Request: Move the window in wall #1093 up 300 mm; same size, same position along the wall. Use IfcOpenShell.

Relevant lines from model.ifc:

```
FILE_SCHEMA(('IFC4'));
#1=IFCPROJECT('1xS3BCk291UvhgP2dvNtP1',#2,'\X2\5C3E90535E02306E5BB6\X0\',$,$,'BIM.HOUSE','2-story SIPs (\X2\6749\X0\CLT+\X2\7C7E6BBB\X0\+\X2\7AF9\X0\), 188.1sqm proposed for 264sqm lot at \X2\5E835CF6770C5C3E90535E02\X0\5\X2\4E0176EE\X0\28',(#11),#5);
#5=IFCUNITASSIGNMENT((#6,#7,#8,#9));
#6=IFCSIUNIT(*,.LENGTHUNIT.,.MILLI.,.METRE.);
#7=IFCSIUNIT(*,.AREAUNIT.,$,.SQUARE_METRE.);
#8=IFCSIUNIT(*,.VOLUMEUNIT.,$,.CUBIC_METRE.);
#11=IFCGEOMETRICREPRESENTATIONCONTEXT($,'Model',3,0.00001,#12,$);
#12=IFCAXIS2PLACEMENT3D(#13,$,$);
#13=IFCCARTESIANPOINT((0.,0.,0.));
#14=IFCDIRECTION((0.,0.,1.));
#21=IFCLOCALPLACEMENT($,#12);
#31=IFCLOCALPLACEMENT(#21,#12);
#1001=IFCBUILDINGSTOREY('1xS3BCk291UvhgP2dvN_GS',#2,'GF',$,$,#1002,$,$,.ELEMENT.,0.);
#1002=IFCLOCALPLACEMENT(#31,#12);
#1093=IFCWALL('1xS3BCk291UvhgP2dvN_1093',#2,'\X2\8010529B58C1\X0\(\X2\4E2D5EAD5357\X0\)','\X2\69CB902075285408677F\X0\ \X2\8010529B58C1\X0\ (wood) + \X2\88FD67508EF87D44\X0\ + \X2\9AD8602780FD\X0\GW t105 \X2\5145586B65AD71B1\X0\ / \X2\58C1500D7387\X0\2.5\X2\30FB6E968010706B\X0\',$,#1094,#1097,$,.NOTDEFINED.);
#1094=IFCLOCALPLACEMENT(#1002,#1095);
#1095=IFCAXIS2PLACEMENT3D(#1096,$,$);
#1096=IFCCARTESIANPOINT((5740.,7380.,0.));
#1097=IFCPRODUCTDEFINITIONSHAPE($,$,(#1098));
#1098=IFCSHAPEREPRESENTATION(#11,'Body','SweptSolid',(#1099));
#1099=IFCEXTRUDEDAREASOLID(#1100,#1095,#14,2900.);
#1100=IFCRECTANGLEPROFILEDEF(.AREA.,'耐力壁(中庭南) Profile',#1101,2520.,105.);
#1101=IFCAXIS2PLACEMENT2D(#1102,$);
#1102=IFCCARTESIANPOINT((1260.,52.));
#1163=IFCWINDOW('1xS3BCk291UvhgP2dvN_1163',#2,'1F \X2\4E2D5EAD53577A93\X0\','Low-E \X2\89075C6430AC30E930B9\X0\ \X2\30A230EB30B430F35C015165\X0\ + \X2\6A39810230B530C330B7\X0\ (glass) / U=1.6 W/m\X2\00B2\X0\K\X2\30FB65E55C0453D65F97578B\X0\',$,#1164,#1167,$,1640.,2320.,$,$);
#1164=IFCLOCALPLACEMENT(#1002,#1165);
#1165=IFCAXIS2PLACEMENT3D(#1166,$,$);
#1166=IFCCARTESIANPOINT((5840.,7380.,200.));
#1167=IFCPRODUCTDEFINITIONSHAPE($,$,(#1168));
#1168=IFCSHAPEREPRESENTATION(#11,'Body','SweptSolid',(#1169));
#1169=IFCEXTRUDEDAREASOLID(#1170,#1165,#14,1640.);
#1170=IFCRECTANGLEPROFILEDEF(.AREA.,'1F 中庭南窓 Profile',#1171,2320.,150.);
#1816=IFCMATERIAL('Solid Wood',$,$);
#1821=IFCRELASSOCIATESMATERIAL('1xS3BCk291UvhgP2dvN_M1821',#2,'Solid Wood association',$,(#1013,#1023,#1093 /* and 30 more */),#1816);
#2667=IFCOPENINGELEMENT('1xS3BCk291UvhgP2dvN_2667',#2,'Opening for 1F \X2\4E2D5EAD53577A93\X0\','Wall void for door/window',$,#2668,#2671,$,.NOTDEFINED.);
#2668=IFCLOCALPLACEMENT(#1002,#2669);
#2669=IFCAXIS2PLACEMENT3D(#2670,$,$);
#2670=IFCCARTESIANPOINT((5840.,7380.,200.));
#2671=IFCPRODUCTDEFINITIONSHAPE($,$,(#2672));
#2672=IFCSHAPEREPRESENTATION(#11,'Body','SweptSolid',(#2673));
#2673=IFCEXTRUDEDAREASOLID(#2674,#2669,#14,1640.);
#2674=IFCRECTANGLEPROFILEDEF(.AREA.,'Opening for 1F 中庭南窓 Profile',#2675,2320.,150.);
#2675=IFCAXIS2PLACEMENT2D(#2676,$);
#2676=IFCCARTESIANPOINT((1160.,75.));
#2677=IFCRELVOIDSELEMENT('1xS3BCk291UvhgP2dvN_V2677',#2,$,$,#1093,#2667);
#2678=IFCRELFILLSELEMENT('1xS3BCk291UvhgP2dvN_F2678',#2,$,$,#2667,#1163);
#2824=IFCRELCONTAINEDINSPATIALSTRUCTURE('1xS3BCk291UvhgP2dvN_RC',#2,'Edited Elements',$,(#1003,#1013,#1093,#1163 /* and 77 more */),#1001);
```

```python
import numpy as np
import ifcopenshell
import ifcopenshell.api.geometry
import ifcopenshell.util.placement
import ifcopenshell.util.unit

model = ifcopenshell.open("model.ifc")
unit_scale = ifcopenshell.util.unit.calculate_unit_scale(model)

window = model.by_id(1163)
opening = window.FillsVoids[0].RelatingOpeningElement
dz = 0.3 / unit_scale

shift = np.array([0.0, 0.0, dz])
# The window is not placed relative to its opening, so move both.
for product in (opening, window):
    matrix = ifcopenshell.util.placement.get_local_placement(product.ObjectPlacement)
    matrix[:3, 3] += shift
    ifcopenshell.api.geometry.edit_object_placement(model, product=product, matrix=matrix, is_si=False)

print(f"moved by {dz * unit_scale:+.3f} m")

model.write("model-out.ifc")
```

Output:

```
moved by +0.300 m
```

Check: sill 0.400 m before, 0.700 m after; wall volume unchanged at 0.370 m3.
